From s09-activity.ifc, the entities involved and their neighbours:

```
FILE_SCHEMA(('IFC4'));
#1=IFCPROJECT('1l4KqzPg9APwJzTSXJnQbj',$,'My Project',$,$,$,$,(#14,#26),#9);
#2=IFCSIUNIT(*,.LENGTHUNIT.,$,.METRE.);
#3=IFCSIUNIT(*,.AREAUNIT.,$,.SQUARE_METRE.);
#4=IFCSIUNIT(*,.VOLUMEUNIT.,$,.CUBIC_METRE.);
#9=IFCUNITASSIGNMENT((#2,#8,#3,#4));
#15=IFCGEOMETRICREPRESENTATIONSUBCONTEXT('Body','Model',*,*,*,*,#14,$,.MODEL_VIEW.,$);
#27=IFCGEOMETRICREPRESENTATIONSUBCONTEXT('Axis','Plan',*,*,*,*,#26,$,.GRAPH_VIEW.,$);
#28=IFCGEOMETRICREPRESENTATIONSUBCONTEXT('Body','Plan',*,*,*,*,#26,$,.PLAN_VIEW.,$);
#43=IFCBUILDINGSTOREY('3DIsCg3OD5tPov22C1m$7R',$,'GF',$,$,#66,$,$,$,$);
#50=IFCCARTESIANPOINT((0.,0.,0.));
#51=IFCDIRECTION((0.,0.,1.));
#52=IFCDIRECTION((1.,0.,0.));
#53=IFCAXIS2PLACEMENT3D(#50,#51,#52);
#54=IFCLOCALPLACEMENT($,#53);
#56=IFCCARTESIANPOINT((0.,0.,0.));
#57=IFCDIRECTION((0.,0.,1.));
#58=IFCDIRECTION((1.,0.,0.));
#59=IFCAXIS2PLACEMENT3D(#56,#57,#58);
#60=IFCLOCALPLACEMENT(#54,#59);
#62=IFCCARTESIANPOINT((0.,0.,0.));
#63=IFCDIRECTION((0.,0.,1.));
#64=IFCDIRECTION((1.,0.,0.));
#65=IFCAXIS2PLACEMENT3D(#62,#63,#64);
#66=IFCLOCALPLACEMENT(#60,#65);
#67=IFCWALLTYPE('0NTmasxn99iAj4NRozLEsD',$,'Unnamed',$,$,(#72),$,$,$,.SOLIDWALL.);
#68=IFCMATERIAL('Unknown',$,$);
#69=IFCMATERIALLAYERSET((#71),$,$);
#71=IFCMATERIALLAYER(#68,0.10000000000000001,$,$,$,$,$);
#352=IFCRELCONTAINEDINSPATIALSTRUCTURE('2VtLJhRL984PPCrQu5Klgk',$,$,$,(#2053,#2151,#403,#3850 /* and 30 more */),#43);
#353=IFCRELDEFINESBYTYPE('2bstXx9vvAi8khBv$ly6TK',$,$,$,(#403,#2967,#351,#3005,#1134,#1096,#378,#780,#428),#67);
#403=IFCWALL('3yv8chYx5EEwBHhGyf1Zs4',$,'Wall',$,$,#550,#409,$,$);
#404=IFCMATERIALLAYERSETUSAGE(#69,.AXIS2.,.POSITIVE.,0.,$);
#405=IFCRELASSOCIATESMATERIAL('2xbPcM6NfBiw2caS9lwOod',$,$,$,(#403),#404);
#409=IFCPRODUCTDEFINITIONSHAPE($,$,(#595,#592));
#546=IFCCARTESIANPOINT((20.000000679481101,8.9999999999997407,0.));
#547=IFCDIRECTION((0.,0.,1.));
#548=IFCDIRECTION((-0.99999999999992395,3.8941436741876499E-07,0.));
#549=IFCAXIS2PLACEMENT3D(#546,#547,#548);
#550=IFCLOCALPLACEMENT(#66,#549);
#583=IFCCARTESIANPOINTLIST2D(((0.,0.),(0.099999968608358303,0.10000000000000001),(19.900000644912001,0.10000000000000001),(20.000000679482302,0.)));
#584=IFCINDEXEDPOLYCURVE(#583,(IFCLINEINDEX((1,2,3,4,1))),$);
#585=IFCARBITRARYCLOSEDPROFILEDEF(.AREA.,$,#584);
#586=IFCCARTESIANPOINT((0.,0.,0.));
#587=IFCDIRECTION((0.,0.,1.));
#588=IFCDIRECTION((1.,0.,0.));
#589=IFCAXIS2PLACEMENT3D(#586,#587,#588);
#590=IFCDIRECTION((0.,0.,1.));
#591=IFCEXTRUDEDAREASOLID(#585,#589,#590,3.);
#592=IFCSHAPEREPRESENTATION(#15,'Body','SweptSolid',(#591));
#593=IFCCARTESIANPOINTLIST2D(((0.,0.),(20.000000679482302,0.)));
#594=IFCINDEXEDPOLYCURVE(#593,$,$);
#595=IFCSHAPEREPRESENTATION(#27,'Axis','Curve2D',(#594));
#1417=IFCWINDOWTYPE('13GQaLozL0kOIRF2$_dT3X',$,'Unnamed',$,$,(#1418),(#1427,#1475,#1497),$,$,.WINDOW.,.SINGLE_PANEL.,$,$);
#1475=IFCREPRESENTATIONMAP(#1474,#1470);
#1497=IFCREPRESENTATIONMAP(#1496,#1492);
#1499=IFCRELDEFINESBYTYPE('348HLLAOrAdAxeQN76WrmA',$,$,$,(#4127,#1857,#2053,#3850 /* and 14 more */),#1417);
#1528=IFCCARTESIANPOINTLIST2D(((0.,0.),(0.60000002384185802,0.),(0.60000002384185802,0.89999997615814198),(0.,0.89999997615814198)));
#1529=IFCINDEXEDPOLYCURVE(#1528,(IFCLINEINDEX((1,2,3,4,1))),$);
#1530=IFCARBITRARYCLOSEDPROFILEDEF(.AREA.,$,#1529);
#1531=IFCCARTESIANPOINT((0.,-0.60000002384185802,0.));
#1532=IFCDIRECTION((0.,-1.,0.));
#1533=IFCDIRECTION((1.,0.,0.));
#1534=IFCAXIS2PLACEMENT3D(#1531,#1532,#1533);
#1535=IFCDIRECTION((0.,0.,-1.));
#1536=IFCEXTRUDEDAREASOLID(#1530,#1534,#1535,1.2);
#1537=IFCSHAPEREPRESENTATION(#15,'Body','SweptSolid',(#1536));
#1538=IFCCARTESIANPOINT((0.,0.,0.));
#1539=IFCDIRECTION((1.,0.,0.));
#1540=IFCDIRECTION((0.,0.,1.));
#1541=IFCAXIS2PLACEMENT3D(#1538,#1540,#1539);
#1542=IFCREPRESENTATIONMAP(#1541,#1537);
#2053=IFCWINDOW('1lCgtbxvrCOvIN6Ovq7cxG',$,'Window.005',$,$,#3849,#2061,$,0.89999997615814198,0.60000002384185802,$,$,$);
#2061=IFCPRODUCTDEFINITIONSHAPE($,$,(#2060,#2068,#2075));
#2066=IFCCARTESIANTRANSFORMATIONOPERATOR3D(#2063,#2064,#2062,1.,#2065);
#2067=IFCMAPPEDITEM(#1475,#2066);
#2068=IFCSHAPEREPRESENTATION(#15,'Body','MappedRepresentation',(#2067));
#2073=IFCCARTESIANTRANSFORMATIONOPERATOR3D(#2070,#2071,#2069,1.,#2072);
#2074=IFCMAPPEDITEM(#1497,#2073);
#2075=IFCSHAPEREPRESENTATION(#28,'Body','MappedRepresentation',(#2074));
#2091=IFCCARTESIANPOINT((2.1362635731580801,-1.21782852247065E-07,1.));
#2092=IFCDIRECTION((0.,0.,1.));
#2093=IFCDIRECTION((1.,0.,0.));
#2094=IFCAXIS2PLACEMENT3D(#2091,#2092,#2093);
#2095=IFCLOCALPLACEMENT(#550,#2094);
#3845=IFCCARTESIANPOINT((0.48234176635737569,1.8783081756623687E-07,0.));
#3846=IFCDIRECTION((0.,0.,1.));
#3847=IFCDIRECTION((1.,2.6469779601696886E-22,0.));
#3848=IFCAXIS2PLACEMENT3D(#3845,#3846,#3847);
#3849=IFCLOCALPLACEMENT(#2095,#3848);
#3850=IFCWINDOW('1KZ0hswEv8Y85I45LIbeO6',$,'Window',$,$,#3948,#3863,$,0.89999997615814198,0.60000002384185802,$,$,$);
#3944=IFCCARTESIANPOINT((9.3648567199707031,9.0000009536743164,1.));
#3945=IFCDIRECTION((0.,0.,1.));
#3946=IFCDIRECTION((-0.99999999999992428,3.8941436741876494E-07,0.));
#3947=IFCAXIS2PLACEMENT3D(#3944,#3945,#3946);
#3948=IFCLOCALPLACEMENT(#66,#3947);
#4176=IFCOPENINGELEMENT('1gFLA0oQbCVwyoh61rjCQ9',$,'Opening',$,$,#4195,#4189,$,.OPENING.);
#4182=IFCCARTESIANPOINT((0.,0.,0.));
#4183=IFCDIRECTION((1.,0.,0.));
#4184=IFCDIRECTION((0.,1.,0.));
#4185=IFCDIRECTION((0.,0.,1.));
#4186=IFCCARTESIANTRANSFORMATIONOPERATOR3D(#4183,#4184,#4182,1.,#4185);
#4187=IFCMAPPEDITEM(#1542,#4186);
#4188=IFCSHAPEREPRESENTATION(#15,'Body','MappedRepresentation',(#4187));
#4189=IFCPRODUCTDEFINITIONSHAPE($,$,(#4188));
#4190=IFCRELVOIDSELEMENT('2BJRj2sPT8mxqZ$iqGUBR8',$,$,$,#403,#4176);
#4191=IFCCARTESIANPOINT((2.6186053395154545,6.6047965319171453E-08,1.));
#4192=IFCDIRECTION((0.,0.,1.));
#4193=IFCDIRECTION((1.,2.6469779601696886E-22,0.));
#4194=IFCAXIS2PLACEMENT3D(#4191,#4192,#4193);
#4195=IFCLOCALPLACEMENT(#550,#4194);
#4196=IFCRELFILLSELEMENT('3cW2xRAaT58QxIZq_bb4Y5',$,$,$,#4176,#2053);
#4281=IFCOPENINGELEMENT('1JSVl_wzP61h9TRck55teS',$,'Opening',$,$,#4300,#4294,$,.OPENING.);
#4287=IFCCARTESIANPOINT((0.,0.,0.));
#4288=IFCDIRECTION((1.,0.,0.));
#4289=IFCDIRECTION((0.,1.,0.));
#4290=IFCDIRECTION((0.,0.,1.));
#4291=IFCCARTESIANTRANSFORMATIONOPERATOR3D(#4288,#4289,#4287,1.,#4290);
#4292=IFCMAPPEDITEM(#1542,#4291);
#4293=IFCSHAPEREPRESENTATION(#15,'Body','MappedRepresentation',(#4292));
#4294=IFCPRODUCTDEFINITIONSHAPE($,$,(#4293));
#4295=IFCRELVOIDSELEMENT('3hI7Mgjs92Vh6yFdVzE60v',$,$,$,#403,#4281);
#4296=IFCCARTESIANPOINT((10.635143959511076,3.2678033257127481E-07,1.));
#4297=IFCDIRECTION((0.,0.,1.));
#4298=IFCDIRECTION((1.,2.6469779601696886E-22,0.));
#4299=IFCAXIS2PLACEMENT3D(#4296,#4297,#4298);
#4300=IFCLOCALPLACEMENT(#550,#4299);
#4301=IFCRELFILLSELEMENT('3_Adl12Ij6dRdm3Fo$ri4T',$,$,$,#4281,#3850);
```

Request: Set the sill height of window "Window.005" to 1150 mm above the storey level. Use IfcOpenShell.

```python
import numpy as np
import ifcopenshell
import ifcopenshell.api.geometry
import ifcopenshell.geom
import ifcopenshell.util.element
import ifcopenshell.util.placement
import ifcopenshell.util.shape
import ifcopenshell.util.unit

model = ifcopenshell.open("s09-activity.ifc")
unit_scale = ifcopenshell.util.unit.calculate_unit_scale(model)

window = model.by_id(2053)
opening = window.FillsVoids[0].RelatingOpeningElement
storey = ifcopenshell.util.element.get_container(window, ifc_class="IfcBuildingStorey")
level = ifcopenshell.util.placement.get_local_placement(storey.ObjectPlacement)[2, 3]

# The opening's origin need not be at the sill, so measure its lowest point.
shape = ifcopenshell.geom.create_shape(ifcopenshell.geom.settings(), opening)
bottom = ifcopenshell.util.shape.get_shape_bottom_elevation(shape, shape.geometry) / unit_scale
dz = level + 1.15 / unit_scale - bottom

shift = np.array([0.0, 0.0, dz])
# The window is not placed relative to its opening, so move both.
for product in (opening, window):
    matrix = ifcopenshell.util.placement.get_local_placement(product.ObjectPlacement)
    matrix[:3, 3] += shift
    ifcopenshell.api.geometry.edit_object_placement(model, product=product, matrix=matrix, is_si=False)

print(f"moved by {dz * unit_scale:+.3f} m")

model.write("s09-activity_updated.ifc")
```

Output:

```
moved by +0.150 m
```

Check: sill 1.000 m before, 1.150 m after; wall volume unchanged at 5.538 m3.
